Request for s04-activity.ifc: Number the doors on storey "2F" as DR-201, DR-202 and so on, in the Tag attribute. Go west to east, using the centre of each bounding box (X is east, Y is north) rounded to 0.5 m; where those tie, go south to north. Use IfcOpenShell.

First a look at what the model holds.

```python
import ifcopenshell
import ifcopenshell.util.element
import ifcopenshell.util.placement

model = ifcopenshell.open("s04-activity.ifc")
print(model.schema)
storey = next(s for s in model.by_type("IfcBuildingStorey") if s.Name == "2F")
doors = [e for e in ifcopenshell.util.element.get_decomposition(storey) if e.is_a("IfcDoor")]
for e in sorted(doors, key=lambda e: e.id()):
    origin = ifcopenshell.util.placement.get_local_placement(e.ObjectPlacement)[:3, 3]
    print(e.id(), e.Tag, e.Name, origin.round(2) + 0.0, sep=" | ")
```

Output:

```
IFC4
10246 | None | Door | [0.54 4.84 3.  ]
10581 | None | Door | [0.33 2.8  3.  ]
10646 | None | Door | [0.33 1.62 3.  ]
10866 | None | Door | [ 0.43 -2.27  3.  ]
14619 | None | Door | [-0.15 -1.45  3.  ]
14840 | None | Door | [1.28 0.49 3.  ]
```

```python
import ifcopenshell
import ifcopenshell.geom
import ifcopenshell.util.element
import ifcopenshell.util.shape

model = ifcopenshell.open("s04-activity.ifc")
settings = ifcopenshell.geom.settings()
settings.set("use-world-coords", True)


def centre(element):
    shape = ifcopenshell.geom.create_shape(settings, element)
    return ifcopenshell.util.shape.get_bbox_centroid(shape.geometry)


storey = next(s for s in model.by_type("IfcBuildingStorey") if s.Name == "2F")
doors = [e for e in ifcopenshell.util.element.get_decomposition(storey) if e.is_a("IfcDoor")]

# Insertion points can sit at a corner or the storey origin, so sort by the geometry (in metres).
centres = {e: centre(e) for e in doors}
doors.sort(key=lambda e: (round(centres[e][0] / 0.5), centres[e][1]))

for i, e in enumerate(doors, start=1):
    number = f"DR-2{i:02d}"
    e.Tag = number
    print(e.id(), number)

model.write("s04-activity-out.ifc")
```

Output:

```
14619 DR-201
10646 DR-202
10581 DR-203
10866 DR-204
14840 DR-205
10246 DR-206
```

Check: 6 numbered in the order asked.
